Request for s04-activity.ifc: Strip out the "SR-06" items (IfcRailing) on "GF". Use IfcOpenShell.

First a look at what the model holds.

```python
import ifcopenshell
import ifcopenshell.util.element

model = ifcopenshell.open("s04-activity.ifc")
print(model.schema)
storey = next(s for s in model.by_type("IfcBuildingStorey") if s.Name == "GF")
railings = [e for e in ifcopenshell.util.element.get_decomposition(storey) if e.is_a("IfcRailing")]
seen = {}
for e in railings:
    element_type = ifcopenshell.util.element.get_type(e)
    name = element_type.Name if element_type not in (None, e) else None
    seen[name] = seen.get(name, 0) + 1
for name, count in sorted(seen.items(), key=str):
    print(count, "x", name)
```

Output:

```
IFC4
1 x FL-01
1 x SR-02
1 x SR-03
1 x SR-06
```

```python
import ifcopenshell
import ifcopenshell.api.root
import ifcopenshell.util.element

model = ifcopenshell.open("s04-activity.ifc")

storey = next(s for s in model.by_type("IfcBuildingStorey") if s.Name == "GF")
railings = [e for e in ifcopenshell.util.element.get_decomposition(storey) if e.is_a("IfcRailing")]
targets = [e for e in railings if (t := ifcopenshell.util.element.get_type(e)) not in (None, e) and t.Name == "SR-06"]

for e in targets:
    ifcopenshell.api.root.remove_product(model, product=e)
print(len(targets), "removed")

model.write("s04-activity_rev.ifc")
```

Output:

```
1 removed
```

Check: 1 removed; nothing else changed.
